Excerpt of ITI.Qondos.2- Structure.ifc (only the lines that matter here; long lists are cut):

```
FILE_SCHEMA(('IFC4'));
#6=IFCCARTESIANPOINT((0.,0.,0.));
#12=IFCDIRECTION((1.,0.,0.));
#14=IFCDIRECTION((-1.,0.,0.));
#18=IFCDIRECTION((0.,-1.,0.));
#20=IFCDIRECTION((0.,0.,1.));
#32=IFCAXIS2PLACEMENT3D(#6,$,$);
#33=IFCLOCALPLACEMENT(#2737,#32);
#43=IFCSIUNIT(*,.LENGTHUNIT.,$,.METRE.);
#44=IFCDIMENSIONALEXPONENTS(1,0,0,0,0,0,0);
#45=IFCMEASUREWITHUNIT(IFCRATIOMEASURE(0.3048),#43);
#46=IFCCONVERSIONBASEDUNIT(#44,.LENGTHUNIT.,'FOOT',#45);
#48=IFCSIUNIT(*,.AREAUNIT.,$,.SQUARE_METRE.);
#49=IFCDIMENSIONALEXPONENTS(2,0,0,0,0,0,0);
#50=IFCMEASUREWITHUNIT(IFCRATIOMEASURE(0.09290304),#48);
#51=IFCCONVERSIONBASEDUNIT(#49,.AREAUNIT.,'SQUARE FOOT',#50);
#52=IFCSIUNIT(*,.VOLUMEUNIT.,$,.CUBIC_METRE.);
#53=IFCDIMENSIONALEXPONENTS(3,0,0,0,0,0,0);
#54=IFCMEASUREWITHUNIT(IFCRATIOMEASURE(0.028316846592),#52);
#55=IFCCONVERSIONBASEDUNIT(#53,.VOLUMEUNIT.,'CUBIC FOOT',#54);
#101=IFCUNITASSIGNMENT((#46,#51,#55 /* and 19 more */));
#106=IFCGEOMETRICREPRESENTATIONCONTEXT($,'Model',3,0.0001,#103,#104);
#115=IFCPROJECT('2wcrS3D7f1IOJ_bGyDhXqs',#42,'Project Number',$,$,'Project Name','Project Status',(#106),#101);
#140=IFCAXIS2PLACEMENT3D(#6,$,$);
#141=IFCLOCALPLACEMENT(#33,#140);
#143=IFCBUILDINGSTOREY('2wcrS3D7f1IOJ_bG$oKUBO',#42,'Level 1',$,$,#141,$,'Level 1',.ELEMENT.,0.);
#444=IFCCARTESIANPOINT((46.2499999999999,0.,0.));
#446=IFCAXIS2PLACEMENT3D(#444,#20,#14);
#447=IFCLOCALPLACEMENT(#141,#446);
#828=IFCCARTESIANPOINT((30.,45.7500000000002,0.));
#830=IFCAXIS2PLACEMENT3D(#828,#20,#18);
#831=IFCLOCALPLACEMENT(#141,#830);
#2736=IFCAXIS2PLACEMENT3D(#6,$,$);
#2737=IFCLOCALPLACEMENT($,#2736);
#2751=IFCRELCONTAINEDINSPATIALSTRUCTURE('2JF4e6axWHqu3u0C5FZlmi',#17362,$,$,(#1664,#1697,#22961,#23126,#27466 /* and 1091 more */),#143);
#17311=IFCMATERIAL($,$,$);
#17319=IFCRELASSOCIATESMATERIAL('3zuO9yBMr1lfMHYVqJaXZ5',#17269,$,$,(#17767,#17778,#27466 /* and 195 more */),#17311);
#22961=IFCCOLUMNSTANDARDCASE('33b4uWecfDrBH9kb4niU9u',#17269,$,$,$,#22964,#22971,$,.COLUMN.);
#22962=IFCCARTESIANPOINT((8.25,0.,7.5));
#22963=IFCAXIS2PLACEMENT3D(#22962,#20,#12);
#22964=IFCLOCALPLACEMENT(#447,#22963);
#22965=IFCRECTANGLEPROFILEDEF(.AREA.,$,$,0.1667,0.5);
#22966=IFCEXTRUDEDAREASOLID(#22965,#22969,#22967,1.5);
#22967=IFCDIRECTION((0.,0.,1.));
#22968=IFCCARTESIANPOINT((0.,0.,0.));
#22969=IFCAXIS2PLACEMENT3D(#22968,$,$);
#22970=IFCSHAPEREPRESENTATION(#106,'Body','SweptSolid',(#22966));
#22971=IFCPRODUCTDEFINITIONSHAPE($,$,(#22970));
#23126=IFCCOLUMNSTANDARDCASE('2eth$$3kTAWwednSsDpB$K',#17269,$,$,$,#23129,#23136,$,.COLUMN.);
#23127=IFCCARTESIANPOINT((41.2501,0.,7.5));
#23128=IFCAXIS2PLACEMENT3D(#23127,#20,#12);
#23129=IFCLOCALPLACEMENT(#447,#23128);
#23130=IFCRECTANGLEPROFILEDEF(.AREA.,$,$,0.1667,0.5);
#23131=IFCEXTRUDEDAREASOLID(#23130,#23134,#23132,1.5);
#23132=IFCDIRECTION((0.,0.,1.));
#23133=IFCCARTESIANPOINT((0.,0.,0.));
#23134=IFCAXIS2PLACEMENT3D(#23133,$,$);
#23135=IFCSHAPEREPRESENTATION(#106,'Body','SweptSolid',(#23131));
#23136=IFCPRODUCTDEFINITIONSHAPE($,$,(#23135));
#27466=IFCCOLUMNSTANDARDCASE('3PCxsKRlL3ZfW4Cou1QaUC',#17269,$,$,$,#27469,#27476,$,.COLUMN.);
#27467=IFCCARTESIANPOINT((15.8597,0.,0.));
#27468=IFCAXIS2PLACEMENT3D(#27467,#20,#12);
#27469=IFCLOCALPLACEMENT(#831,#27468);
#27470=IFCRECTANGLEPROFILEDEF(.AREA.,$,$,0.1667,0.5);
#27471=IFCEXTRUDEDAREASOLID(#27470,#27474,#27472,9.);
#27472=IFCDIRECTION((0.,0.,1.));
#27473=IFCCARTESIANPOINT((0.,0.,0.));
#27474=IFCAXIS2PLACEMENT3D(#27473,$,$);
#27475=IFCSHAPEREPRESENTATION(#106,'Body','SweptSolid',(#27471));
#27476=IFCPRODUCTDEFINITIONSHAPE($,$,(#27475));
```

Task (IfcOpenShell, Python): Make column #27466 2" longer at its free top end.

```python
import ifcopenshell
import ifcopenshell.util.unit

model = ifcopenshell.open("ITI.Qondos.2- Structure.ifc")
unit_scale = ifcopenshell.util.unit.calculate_unit_scale(model)

member = model.by_id(27466)
change = 2 * 0.0254 / unit_scale

# The extrusion runs towards the end named, so only its depth changes.
body = next(r for r in member.Representation.Representations if r.RepresentationIdentifier == "Body")
solid = body.Items[0]
old_length = solid.Depth
solid.Depth += change

print(f"length {old_length:g} -> {solid.Depth:g}")

model.write("ITI.Qondos.2- Structure-out.ifc")
```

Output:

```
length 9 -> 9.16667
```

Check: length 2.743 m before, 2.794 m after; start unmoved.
